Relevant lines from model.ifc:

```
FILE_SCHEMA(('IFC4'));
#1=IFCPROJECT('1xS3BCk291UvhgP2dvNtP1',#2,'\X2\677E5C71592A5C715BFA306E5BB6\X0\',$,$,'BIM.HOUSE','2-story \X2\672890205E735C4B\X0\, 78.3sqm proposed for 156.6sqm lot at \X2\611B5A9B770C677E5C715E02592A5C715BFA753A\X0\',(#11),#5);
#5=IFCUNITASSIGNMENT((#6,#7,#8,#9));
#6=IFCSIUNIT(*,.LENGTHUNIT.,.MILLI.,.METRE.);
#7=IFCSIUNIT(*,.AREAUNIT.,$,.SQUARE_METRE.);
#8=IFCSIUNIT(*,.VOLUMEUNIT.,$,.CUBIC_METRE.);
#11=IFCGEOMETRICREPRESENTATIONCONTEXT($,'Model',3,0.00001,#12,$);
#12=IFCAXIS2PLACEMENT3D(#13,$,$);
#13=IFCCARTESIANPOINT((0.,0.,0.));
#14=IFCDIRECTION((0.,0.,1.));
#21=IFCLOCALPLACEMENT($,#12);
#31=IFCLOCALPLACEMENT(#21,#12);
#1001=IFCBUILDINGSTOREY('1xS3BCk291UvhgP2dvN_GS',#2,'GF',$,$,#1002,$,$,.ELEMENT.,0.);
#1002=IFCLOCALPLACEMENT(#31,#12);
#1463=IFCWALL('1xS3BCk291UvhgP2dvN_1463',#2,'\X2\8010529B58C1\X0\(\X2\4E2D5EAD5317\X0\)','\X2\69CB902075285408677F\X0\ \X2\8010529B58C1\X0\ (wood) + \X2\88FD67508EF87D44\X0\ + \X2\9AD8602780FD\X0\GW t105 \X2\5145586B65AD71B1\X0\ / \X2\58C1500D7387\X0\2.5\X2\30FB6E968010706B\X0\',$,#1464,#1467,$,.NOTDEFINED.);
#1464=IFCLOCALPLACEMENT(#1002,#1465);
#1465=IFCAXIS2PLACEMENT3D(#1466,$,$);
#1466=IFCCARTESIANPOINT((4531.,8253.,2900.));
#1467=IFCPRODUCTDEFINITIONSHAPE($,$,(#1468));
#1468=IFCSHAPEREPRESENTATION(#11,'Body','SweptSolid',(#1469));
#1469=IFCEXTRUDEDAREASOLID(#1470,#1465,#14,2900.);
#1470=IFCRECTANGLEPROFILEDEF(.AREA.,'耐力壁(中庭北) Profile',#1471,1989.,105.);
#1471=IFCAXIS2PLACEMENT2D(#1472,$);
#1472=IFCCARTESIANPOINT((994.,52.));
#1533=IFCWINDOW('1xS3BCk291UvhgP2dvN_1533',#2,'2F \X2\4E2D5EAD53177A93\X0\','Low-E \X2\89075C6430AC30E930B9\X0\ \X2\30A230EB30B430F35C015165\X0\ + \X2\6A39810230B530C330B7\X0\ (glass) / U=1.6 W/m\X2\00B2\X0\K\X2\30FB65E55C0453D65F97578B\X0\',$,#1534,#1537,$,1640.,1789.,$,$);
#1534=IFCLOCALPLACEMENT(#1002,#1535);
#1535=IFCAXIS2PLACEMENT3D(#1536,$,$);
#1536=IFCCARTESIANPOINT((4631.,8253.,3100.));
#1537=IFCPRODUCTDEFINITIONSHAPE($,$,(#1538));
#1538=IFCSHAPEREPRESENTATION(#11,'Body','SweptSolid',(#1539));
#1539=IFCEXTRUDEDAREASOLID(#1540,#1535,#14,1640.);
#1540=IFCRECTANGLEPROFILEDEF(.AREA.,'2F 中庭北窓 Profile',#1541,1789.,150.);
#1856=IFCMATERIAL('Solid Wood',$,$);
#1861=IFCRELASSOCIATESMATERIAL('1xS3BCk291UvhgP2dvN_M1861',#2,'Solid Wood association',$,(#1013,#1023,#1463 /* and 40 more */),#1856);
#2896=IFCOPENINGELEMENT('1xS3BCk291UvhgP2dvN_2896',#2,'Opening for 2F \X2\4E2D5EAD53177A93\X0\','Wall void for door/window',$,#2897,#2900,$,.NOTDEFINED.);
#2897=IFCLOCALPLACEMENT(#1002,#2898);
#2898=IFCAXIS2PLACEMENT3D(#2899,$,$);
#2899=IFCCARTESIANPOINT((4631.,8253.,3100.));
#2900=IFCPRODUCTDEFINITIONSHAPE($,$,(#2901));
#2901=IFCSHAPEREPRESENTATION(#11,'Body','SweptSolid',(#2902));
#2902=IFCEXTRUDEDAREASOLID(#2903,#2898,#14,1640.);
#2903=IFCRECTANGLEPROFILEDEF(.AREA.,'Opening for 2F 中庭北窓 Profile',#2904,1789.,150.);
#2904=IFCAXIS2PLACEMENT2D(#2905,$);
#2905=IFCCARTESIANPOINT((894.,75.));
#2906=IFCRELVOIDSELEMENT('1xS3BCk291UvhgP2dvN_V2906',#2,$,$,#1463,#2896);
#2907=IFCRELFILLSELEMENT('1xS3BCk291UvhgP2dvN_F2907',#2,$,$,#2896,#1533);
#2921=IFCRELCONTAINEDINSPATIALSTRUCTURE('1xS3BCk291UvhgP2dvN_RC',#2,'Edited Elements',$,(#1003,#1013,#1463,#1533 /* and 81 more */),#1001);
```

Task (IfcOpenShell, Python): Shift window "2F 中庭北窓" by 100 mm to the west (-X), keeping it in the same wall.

```python
import ifcopenshell
import ifcopenshell.api.geometry
import ifcopenshell.util.placement
import ifcopenshell.util.unit

model = ifcopenshell.open("model.ifc")
unit_scale = ifcopenshell.util.unit.calculate_unit_scale(model)

window = model.by_guid("1xS3BCk291UvhgP2dvN_1533")
opening = window.FillsVoids[0].RelatingOpeningElement
wall = opening.VoidsElements[0].RelatingBuildingElement

wall_matrix = ifcopenshell.util.placement.get_local_placement(wall.ObjectPlacement)
shift = wall_matrix[:3, 0] * -0.1 / unit_scale
before = ifcopenshell.util.placement.get_local_placement(window.ObjectPlacement)[:3, 3].copy()

# The window is not placed relative to its opening, so move both.
for product in (opening, window):
    matrix = ifcopenshell.util.placement.get_local_placement(product.ObjectPlacement)
    matrix[:3, 3] += shift
    ifcopenshell.api.geometry.edit_object_placement(model, product=product, matrix=matrix, is_si=False)

after = ifcopenshell.util.placement.get_local_placement(window.ObjectPlacement)[:3, 3]
print("window moved by", (after - before).round(3) + 0.0)

model.write("model_edited.ifc")
```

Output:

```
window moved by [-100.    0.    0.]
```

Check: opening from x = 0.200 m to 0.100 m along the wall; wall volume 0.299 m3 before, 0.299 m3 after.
